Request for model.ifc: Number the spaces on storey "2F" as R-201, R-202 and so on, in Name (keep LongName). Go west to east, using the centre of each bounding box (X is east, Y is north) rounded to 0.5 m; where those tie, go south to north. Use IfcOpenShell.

First a look at what the model holds.

```python
import ifcopenshell
import ifcopenshell.util.element
import ifcopenshell.util.placement

model = ifcopenshell.open("model.ifc")
print(model.schema)
storey = next(s for s in model.by_type("IfcBuildingStorey") if s.Name == "2F")
spaces = [e for e in ifcopenshell.util.element.get_decomposition(storey) if e.is_a("IfcSpace")]
for e in sorted(spaces, key=lambda e: e.id()):
    origin = ifcopenshell.util.placement.get_local_placement(e.ObjectPlacement)[:3, 3]
    print(e.id(), e.Name, e.LongName, origin.round(2) + 0.0, sep=" | ")
```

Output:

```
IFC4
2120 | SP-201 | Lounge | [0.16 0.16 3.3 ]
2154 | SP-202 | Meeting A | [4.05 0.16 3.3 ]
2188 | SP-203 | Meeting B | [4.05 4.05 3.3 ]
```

```python
import ifcopenshell
import ifcopenshell.geom
import ifcopenshell.util.element
import ifcopenshell.util.shape

model = ifcopenshell.open("model.ifc")
settings = ifcopenshell.geom.settings()
settings.set("use-world-coords", True)


def centre(element):
    shape = ifcopenshell.geom.create_shape(settings, element)
    return ifcopenshell.util.shape.get_bbox_centroid(shape.geometry)


storey = next(s for s in model.by_type("IfcBuildingStorey") if s.Name == "2F")
spaces = [e for e in ifcopenshell.util.element.get_decomposition(storey) if e.is_a("IfcSpace")]

# Insertion points can sit at a corner or the storey origin, so sort by the geometry (in metres).
centres = {e: centre(e) for e in spaces}
spaces.sort(key=lambda e: (round(centres[e][0] / 0.5), centres[e][1]))

for i, e in enumerate(spaces, start=1):
    number = f"R-2{i:02d}"
    e.Name = number
    print(e.id(), number)

model.write("model_updated.ifc")
```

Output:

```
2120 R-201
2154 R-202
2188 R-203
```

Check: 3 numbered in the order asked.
